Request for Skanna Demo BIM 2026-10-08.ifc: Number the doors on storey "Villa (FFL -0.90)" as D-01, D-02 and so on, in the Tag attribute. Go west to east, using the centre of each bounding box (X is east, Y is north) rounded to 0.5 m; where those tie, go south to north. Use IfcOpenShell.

First a look at what the model holds.

```python
import ifcopenshell
import ifcopenshell.util.element
import ifcopenshell.util.placement

model = ifcopenshell.open("Skanna Demo BIM 2026-10-08.ifc")
print(model.schema)
storey = next(s for s in model.by_type("IfcBuildingStorey") if s.Name == "Villa (FFL -0.90)")
doors = [e for e in ifcopenshell.util.element.get_decomposition(storey) if e.is_a("IfcDoor")]
for e in sorted(doors, key=lambda e: e.id()):
    origin = ifcopenshell.util.placement.get_local_placement(e.ObjectPlacement)[:3, 3]
    print(e.id(), e.Tag, e.Name, origin.round(2) + 0.0, sep=" | ")
```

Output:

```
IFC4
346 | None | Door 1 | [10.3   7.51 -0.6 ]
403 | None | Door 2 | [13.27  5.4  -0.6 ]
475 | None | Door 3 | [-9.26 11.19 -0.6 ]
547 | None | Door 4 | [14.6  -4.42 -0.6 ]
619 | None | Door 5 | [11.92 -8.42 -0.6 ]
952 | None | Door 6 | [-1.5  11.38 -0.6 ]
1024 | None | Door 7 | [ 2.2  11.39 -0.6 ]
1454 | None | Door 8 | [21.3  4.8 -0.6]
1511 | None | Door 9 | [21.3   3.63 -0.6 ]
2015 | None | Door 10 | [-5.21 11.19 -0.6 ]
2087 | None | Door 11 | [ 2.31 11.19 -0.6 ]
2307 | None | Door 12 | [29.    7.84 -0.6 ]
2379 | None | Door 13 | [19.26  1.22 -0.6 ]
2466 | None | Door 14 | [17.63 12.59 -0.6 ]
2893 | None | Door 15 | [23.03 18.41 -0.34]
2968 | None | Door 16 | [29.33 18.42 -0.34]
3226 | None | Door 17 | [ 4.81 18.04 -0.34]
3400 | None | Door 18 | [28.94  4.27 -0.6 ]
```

```python
import ifcopenshell
import ifcopenshell.geom
import ifcopenshell.util.element
import ifcopenshell.util.shape

model = ifcopenshell.open("Skanna Demo BIM 2026-10-08.ifc")
settings = ifcopenshell.geom.settings()
settings.set("use-world-coords", True)


def centre(element):
    shape = ifcopenshell.geom.create_shape(settings, element)
    return ifcopenshell.util.shape.get_bbox_centroid(shape.geometry)


storey = next(s for s in model.by_type("IfcBuildingStorey") if s.Name == "Villa (FFL -0.90)")
doors = [e for e in ifcopenshell.util.element.get_decomposition(storey) if e.is_a("IfcDoor")]

# Insertion points can sit at a corner or the storey origin, so sort by the geometry (in metres).
centres = {e: centre(e) for e in doors}
doors.sort(key=lambda e: (round(centres[e][0] / 0.5), centres[e][1]))

for i, e in enumerate(doors, start=1):
    number = f"D-{i:02d}"
    e.Tag = number
    print(e.id(), number)

model.write("Skanna Demo BIM 2026-10-08_updated.ifc")
```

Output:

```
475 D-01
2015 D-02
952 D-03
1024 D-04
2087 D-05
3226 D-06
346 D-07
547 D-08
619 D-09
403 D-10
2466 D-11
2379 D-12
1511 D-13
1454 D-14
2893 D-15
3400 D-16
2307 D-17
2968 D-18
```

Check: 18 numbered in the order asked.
